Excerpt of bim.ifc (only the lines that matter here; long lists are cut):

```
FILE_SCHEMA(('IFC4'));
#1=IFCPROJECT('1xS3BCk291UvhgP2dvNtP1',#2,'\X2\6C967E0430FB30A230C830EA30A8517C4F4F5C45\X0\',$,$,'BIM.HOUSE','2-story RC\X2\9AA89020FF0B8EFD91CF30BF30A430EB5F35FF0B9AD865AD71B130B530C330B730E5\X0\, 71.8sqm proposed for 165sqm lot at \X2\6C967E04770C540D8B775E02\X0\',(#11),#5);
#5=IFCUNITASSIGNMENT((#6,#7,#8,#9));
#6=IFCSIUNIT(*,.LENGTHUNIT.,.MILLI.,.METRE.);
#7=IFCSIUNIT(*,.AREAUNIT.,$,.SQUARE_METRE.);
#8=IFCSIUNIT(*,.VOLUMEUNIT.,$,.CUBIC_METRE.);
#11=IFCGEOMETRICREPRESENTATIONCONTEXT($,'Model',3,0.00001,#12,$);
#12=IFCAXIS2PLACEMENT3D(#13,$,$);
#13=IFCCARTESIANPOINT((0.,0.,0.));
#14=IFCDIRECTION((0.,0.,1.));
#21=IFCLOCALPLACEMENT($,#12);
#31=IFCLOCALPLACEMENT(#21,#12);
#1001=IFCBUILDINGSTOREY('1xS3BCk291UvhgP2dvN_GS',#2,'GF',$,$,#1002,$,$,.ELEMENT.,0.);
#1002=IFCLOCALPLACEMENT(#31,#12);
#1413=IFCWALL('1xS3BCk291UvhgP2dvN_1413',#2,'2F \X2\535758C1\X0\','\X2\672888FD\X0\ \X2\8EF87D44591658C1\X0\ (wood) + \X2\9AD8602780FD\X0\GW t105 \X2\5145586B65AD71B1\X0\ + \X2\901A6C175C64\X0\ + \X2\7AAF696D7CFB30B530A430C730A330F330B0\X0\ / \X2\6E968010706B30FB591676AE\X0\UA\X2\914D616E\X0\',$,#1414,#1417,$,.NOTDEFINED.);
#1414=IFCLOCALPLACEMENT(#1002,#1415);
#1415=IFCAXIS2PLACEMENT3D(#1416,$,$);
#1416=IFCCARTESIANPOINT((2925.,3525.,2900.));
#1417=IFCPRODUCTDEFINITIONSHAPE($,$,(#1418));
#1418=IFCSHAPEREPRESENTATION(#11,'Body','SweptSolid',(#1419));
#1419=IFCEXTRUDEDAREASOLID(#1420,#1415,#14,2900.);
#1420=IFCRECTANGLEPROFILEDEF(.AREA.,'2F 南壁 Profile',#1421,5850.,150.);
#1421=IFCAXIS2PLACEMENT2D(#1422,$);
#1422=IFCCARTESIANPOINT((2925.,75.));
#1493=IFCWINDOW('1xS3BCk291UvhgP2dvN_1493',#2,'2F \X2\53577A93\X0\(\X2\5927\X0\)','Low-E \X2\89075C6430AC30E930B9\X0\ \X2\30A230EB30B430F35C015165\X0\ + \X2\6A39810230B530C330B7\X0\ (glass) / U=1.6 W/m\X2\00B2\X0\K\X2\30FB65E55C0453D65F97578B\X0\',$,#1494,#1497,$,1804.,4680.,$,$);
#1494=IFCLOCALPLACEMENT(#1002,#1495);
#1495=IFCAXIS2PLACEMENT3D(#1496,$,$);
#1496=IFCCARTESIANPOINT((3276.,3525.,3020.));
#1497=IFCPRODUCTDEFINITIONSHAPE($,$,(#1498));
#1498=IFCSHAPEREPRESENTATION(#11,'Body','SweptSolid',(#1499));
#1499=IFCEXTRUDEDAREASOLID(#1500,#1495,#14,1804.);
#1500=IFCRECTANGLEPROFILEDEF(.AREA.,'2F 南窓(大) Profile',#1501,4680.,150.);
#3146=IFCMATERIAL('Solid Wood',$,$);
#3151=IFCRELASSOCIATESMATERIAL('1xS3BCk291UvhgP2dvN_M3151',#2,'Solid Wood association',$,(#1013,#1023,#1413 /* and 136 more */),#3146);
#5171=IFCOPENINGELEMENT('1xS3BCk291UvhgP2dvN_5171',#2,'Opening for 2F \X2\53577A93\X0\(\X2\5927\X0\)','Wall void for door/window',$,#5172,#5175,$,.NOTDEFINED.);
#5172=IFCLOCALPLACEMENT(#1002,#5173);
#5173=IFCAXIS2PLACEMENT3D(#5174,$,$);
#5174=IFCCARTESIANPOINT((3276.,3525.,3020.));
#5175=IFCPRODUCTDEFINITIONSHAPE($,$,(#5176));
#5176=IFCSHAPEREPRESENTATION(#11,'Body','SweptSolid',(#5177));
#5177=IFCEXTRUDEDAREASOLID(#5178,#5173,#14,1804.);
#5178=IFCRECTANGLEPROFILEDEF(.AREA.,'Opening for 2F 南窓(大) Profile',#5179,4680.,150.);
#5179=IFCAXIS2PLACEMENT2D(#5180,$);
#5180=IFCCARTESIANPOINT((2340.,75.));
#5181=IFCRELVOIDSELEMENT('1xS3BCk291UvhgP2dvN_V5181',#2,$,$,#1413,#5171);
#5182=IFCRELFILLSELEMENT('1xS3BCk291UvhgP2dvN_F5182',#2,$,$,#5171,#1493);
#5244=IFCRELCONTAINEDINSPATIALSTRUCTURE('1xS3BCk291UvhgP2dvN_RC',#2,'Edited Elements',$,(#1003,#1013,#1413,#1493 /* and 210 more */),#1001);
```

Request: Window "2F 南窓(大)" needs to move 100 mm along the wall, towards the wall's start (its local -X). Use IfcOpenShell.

```python
import ifcopenshell
import ifcopenshell.api.geometry
import ifcopenshell.util.placement

model = ifcopenshell.open("bim.ifc")

window = model.by_id(1493)
opening = window.FillsVoids[0].RelatingOpeningElement
wall = opening.VoidsElements[0].RelatingBuildingElement

wall_matrix = ifcopenshell.util.placement.get_local_placement(wall.ObjectPlacement)
shift = wall_matrix[:3, 0] * -100.0
before = ifcopenshell.util.placement.get_local_placement(window.ObjectPlacement)[:3, 3].copy()

# The window is not placed relative to its opening, so move both.
for product in (opening, window):
    matrix = ifcopenshell.util.placement.get_local_placement(product.ObjectPlacement)
    matrix[:3, 3] += shift
    ifcopenshell.api.geometry.edit_object_placement(model, product=product, matrix=matrix, is_si=False)

after = ifcopenshell.util.placement.get_local_placement(window.ObjectPlacement)[:3, 3]
print("window moved by", (after - before).round(3) + 0.0)

model.write("bim_rev.ifc")
```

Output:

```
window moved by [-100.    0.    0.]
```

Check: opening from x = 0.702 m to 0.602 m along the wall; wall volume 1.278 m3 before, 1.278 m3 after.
